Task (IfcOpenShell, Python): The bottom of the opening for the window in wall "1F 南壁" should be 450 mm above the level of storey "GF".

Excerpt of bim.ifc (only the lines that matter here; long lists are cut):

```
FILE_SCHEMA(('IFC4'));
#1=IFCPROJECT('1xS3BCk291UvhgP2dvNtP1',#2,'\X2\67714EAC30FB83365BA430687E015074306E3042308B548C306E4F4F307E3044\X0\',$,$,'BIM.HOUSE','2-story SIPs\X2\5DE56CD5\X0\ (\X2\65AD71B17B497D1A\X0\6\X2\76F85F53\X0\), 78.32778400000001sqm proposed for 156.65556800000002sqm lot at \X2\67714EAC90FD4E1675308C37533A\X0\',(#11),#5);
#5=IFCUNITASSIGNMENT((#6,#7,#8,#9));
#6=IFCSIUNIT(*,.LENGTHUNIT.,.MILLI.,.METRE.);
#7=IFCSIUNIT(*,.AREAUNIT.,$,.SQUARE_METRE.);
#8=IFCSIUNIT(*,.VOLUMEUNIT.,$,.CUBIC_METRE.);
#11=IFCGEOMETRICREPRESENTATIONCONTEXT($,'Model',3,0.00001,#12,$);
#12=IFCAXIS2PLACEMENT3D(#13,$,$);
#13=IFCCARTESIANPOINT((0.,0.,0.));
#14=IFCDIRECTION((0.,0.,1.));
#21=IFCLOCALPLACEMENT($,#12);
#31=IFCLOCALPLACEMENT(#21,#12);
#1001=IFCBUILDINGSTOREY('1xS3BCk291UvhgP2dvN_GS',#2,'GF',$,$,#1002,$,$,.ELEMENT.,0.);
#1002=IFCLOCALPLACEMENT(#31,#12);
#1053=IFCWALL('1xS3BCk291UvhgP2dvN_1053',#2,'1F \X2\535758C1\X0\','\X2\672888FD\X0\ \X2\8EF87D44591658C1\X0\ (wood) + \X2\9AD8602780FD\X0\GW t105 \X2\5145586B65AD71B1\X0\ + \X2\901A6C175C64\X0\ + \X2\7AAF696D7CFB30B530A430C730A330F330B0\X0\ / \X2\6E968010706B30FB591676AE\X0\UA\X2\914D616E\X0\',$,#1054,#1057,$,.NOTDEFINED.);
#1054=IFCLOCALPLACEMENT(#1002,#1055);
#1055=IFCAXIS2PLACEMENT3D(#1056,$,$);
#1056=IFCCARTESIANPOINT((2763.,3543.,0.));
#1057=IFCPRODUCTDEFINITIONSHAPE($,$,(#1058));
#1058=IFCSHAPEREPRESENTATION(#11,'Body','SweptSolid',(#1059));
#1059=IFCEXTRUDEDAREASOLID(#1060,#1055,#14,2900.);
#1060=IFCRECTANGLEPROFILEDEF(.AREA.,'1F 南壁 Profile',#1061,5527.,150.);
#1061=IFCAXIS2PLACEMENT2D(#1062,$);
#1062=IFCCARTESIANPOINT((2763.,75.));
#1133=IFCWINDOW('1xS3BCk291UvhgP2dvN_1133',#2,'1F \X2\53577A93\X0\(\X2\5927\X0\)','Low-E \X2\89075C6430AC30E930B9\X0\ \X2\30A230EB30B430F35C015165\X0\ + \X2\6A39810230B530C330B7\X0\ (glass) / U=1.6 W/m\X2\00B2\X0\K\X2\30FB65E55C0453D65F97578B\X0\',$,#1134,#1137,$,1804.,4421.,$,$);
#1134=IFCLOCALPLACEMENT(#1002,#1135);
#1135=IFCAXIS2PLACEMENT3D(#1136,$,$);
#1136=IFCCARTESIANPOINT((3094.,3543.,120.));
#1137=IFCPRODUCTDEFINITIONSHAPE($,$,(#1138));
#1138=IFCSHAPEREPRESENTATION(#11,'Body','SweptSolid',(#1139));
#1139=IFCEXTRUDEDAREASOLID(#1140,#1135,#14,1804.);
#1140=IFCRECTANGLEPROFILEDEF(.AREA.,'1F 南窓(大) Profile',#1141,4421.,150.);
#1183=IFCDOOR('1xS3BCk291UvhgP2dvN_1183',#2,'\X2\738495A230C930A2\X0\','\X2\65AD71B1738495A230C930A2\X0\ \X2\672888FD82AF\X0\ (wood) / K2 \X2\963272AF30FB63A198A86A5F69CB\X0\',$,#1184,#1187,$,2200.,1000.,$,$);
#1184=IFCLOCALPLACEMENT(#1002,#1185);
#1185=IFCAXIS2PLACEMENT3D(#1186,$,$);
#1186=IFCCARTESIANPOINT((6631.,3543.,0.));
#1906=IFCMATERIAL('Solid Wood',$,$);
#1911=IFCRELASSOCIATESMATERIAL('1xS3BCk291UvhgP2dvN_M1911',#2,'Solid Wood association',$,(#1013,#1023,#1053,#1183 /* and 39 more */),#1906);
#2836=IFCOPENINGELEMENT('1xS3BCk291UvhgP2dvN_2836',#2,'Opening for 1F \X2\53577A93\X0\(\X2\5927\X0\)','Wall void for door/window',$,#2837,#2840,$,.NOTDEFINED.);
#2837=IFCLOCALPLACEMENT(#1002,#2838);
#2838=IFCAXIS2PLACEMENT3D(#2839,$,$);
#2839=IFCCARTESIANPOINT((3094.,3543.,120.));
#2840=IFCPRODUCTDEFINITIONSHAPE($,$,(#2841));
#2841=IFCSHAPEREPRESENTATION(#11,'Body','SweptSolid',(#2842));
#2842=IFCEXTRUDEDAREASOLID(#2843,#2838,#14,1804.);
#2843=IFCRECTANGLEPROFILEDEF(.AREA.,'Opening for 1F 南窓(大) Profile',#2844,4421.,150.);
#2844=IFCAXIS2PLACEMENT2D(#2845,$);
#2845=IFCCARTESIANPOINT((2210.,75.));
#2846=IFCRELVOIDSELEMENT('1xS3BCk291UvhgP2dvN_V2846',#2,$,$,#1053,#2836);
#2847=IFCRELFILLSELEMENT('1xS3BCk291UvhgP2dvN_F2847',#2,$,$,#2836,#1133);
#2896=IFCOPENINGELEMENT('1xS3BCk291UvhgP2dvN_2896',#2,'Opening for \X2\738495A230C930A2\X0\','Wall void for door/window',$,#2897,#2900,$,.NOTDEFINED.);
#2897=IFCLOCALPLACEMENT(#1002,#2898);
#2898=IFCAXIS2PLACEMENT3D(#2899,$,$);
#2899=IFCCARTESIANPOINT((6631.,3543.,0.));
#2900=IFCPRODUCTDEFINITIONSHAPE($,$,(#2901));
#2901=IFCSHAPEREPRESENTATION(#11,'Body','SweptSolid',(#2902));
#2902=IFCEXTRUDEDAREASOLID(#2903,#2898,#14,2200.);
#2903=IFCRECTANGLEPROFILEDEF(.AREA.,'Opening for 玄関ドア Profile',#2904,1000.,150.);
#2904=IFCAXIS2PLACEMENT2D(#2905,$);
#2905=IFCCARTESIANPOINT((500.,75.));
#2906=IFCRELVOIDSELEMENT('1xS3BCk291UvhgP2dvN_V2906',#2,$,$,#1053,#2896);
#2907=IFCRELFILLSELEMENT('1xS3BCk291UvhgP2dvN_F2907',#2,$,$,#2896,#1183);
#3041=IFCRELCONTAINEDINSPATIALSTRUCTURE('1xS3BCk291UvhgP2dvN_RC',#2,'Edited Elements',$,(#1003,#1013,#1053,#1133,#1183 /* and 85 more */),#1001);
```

```python
import numpy as np
import ifcopenshell
import ifcopenshell.api.geometry
import ifcopenshell.geom
import ifcopenshell.util.element
import ifcopenshell.util.placement
import ifcopenshell.util.shape
import ifcopenshell.util.unit

model = ifcopenshell.open("bim.ifc")
unit_scale = ifcopenshell.util.unit.calculate_unit_scale(model)

window = model.by_guid("1xS3BCk291UvhgP2dvN_1133")
opening = window.FillsVoids[0].RelatingOpeningElement
storey = ifcopenshell.util.element.get_container(window, ifc_class="IfcBuildingStorey")
level = ifcopenshell.util.placement.get_local_placement(storey.ObjectPlacement)[2, 3]

# The opening's origin need not be at the sill, so measure its lowest point.
shape = ifcopenshell.geom.create_shape(ifcopenshell.geom.settings(), opening)
bottom = ifcopenshell.util.shape.get_shape_bottom_elevation(shape, shape.geometry) / unit_scale
dz = level + 450.0 - bottom

shift = np.array([0.0, 0.0, dz])
# The window is not placed relative to its opening, so move both.
for product in (opening, window):
    matrix = ifcopenshell.util.placement.get_local_placement(product.ObjectPlacement)
    matrix[:3, 3] += shift
    ifcopenshell.api.geometry.edit_object_placement(model, product=product, matrix=matrix, is_si=False)

print(f"moved by {dz * unit_scale:+.3f} m")

model.write("bim_v2.ifc")
```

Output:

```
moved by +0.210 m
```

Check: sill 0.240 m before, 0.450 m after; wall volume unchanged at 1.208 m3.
